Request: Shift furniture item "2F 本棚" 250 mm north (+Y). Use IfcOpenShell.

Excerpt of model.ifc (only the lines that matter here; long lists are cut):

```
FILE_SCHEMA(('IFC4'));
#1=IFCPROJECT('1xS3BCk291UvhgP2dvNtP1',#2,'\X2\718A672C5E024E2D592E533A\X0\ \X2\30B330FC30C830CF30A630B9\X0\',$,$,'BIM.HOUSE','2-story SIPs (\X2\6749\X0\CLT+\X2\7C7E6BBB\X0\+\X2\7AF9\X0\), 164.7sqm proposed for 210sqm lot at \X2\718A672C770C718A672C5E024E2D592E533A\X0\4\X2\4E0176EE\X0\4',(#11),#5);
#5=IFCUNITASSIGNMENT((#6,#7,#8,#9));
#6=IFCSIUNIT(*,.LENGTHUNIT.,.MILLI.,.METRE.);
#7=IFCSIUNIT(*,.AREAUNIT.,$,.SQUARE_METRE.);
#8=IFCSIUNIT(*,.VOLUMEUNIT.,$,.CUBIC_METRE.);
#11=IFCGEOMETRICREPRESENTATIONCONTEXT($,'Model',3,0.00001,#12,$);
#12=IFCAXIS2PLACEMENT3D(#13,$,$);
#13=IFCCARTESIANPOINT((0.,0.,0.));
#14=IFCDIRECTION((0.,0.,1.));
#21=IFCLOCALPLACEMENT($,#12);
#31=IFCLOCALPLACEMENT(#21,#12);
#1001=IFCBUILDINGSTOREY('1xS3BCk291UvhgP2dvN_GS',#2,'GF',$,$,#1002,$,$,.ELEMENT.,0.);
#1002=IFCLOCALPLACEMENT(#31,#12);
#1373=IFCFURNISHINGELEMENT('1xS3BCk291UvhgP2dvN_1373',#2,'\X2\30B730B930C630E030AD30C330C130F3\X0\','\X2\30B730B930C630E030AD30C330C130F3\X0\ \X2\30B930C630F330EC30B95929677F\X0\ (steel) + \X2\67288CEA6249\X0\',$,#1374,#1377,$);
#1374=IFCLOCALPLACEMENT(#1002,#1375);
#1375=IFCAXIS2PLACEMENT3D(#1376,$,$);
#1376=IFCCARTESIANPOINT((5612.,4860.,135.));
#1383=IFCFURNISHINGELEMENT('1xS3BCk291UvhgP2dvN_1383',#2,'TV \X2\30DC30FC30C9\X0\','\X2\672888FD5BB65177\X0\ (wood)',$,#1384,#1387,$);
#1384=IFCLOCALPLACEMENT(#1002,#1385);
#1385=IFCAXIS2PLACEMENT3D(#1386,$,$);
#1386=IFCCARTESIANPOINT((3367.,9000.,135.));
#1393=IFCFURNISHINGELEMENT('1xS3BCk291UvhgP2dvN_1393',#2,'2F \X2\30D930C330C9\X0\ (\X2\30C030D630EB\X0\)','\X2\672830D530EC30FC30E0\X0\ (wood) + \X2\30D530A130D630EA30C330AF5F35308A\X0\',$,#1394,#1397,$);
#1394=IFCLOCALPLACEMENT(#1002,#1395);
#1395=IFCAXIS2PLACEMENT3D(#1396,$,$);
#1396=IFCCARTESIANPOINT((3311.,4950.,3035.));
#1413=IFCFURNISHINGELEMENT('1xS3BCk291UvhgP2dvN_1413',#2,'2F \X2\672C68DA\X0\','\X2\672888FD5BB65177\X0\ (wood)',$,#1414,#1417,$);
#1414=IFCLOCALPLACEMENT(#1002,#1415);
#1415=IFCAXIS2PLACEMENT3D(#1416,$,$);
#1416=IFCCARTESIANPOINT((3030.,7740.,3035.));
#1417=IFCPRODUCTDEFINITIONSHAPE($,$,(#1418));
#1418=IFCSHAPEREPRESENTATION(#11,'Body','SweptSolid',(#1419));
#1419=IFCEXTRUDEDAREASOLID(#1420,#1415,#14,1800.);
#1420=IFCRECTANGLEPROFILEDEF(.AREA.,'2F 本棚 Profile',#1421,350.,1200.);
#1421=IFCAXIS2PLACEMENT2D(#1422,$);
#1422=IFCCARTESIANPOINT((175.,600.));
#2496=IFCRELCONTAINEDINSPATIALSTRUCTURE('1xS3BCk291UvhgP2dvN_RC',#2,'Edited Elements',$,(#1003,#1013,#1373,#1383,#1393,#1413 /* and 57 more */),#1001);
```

```python
import ifcopenshell
import ifcopenshell.api.geometry
import ifcopenshell.util.placement
import ifcopenshell.util.unit

model = ifcopenshell.open("model.ifc")
unit_scale = ifcopenshell.util.unit.calculate_unit_scale(model)

item = model.by_guid("1xS3BCk291UvhgP2dvN_1413")
matrix = ifcopenshell.util.placement.get_local_placement(item.ObjectPlacement)
matrix[1, 3] += 0.25 / unit_scale
ifcopenshell.api.geometry.edit_object_placement(model, product=item, matrix=matrix, is_si=False)

print(ifcopenshell.util.placement.get_local_placement(item.ObjectPlacement).round(3) + 0.0)

model.write("model_updated.ifc")
```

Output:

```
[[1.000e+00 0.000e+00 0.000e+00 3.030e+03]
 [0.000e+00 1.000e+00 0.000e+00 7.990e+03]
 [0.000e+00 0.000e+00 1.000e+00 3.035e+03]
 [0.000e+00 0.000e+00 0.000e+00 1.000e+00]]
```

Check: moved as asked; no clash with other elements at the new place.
